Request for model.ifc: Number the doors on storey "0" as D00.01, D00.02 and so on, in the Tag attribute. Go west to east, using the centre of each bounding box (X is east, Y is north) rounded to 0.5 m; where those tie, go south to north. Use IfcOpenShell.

First a look at what the model holds.

```python
import ifcopenshell
import ifcopenshell.util.element
import ifcopenshell.util.placement

model = ifcopenshell.open("model.ifc")
print(model.schema)
storey = next(s for s in model.by_type("IfcBuildingStorey") if s.Name == "0")
doors = [e for e in ifcopenshell.util.element.get_decomposition(storey) if e.is_a("IfcDoor")]
for e in sorted(doors, key=lambda e: e.id()):
    origin = ifcopenshell.util.placement.get_local_placement(e.ObjectPlacement)[:3, 3]
    print(e.id(), e.Tag, e.Name, origin.round(2) + 0.0, sep=" | ")
```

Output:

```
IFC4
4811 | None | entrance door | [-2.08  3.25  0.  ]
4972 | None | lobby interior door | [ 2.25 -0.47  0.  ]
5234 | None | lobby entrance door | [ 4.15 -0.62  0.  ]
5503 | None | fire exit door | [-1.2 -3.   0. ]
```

```python
import ifcopenshell
import ifcopenshell.geom
import ifcopenshell.util.element
import ifcopenshell.util.shape

model = ifcopenshell.open("model.ifc")
settings = ifcopenshell.geom.settings()
settings.set("use-world-coords", True)


def centre(element):
    shape = ifcopenshell.geom.create_shape(settings, element)
    return ifcopenshell.util.shape.get_bbox_centroid(shape.geometry)


storey = next(s for s in model.by_type("IfcBuildingStorey") if s.Name == "0")
doors = [e for e in ifcopenshell.util.element.get_decomposition(storey) if e.is_a("IfcDoor")]

# Insertion points can sit at a corner or the storey origin, so sort by the geometry (in metres).
centres = {e: centre(e) for e in doors}
doors.sort(key=lambda e: (round(centres[e][0] / 0.5), centres[e][1]))

for i, e in enumerate(doors, start=1):
    number = f"D00.{i:02d}"
    e.Tag = number
    print(e.id(), number)

model.write("model_v2.ifc")
```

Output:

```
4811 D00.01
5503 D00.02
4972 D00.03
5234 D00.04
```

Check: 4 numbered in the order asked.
